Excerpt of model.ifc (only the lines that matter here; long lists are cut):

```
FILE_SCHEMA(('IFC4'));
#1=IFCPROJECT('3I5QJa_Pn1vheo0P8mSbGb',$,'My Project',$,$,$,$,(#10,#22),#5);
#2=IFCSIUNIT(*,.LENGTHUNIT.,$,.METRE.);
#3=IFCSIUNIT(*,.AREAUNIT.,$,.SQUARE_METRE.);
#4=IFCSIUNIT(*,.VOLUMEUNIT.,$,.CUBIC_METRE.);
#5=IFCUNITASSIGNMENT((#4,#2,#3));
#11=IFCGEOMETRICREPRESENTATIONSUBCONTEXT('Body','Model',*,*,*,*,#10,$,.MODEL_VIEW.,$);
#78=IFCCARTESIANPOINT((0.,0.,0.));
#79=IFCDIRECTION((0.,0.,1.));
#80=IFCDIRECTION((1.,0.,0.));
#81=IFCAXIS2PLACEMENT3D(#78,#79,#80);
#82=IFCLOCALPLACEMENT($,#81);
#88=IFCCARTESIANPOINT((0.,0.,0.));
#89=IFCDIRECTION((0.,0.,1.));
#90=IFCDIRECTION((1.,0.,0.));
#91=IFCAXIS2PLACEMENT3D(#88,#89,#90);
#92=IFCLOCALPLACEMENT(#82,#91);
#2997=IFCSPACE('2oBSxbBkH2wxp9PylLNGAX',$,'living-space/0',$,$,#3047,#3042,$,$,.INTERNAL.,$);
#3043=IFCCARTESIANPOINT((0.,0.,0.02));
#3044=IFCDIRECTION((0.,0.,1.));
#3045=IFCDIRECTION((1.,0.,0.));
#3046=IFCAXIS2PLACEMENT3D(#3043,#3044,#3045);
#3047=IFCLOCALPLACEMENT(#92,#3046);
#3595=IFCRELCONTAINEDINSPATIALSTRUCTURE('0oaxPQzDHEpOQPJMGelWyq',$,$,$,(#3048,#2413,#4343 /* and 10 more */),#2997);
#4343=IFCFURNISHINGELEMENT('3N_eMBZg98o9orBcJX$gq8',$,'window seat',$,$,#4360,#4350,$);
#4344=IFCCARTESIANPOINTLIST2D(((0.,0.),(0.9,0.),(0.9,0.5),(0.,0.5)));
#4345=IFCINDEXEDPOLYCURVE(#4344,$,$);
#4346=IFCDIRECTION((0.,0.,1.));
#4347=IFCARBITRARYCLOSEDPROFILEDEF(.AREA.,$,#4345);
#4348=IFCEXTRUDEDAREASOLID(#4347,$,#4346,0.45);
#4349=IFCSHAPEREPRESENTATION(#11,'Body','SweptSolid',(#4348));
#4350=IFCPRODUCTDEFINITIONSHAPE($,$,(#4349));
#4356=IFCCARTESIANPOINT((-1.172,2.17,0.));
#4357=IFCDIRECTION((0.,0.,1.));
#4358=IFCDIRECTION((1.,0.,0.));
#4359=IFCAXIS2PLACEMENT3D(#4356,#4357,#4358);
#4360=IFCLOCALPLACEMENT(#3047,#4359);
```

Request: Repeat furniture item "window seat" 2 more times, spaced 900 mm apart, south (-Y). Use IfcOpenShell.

```python
import numpy as np
import ifcopenshell
import ifcopenshell.api.geometry
import ifcopenshell.api.root
import ifcopenshell.util.element
import ifcopenshell.util.placement
import ifcopenshell.util.unit

model = ifcopenshell.open("model.ifc")
unit_scale = ifcopenshell.util.unit.calculate_unit_scale(model)

source = model.by_id(4343)
base = ifcopenshell.util.placement.get_local_placement(source.ObjectPlacement)
step = np.array([0.0, -1.0, 0.0]) * 0.9 / unit_scale

for i in range(1, 3):
    copy = ifcopenshell.api.root.copy_class(model, product=source)
    copy.Representation = ifcopenshell.util.element.copy_deep(
        model, source.Representation, exclude=["IfcGeometricRepresentationContext", "IfcRepresentationMap"]
    )
    matrix = base.copy()
    matrix[:3, 3] += i * step
    print("added at", matrix[:3, 3].round(3) + 0.0)
    ifcopenshell.api.geometry.edit_object_placement(model, product=copy, matrix=matrix, is_si=False)

model.write("model_rev.ifc")
```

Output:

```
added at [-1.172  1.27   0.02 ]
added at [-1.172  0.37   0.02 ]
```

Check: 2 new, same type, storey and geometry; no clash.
